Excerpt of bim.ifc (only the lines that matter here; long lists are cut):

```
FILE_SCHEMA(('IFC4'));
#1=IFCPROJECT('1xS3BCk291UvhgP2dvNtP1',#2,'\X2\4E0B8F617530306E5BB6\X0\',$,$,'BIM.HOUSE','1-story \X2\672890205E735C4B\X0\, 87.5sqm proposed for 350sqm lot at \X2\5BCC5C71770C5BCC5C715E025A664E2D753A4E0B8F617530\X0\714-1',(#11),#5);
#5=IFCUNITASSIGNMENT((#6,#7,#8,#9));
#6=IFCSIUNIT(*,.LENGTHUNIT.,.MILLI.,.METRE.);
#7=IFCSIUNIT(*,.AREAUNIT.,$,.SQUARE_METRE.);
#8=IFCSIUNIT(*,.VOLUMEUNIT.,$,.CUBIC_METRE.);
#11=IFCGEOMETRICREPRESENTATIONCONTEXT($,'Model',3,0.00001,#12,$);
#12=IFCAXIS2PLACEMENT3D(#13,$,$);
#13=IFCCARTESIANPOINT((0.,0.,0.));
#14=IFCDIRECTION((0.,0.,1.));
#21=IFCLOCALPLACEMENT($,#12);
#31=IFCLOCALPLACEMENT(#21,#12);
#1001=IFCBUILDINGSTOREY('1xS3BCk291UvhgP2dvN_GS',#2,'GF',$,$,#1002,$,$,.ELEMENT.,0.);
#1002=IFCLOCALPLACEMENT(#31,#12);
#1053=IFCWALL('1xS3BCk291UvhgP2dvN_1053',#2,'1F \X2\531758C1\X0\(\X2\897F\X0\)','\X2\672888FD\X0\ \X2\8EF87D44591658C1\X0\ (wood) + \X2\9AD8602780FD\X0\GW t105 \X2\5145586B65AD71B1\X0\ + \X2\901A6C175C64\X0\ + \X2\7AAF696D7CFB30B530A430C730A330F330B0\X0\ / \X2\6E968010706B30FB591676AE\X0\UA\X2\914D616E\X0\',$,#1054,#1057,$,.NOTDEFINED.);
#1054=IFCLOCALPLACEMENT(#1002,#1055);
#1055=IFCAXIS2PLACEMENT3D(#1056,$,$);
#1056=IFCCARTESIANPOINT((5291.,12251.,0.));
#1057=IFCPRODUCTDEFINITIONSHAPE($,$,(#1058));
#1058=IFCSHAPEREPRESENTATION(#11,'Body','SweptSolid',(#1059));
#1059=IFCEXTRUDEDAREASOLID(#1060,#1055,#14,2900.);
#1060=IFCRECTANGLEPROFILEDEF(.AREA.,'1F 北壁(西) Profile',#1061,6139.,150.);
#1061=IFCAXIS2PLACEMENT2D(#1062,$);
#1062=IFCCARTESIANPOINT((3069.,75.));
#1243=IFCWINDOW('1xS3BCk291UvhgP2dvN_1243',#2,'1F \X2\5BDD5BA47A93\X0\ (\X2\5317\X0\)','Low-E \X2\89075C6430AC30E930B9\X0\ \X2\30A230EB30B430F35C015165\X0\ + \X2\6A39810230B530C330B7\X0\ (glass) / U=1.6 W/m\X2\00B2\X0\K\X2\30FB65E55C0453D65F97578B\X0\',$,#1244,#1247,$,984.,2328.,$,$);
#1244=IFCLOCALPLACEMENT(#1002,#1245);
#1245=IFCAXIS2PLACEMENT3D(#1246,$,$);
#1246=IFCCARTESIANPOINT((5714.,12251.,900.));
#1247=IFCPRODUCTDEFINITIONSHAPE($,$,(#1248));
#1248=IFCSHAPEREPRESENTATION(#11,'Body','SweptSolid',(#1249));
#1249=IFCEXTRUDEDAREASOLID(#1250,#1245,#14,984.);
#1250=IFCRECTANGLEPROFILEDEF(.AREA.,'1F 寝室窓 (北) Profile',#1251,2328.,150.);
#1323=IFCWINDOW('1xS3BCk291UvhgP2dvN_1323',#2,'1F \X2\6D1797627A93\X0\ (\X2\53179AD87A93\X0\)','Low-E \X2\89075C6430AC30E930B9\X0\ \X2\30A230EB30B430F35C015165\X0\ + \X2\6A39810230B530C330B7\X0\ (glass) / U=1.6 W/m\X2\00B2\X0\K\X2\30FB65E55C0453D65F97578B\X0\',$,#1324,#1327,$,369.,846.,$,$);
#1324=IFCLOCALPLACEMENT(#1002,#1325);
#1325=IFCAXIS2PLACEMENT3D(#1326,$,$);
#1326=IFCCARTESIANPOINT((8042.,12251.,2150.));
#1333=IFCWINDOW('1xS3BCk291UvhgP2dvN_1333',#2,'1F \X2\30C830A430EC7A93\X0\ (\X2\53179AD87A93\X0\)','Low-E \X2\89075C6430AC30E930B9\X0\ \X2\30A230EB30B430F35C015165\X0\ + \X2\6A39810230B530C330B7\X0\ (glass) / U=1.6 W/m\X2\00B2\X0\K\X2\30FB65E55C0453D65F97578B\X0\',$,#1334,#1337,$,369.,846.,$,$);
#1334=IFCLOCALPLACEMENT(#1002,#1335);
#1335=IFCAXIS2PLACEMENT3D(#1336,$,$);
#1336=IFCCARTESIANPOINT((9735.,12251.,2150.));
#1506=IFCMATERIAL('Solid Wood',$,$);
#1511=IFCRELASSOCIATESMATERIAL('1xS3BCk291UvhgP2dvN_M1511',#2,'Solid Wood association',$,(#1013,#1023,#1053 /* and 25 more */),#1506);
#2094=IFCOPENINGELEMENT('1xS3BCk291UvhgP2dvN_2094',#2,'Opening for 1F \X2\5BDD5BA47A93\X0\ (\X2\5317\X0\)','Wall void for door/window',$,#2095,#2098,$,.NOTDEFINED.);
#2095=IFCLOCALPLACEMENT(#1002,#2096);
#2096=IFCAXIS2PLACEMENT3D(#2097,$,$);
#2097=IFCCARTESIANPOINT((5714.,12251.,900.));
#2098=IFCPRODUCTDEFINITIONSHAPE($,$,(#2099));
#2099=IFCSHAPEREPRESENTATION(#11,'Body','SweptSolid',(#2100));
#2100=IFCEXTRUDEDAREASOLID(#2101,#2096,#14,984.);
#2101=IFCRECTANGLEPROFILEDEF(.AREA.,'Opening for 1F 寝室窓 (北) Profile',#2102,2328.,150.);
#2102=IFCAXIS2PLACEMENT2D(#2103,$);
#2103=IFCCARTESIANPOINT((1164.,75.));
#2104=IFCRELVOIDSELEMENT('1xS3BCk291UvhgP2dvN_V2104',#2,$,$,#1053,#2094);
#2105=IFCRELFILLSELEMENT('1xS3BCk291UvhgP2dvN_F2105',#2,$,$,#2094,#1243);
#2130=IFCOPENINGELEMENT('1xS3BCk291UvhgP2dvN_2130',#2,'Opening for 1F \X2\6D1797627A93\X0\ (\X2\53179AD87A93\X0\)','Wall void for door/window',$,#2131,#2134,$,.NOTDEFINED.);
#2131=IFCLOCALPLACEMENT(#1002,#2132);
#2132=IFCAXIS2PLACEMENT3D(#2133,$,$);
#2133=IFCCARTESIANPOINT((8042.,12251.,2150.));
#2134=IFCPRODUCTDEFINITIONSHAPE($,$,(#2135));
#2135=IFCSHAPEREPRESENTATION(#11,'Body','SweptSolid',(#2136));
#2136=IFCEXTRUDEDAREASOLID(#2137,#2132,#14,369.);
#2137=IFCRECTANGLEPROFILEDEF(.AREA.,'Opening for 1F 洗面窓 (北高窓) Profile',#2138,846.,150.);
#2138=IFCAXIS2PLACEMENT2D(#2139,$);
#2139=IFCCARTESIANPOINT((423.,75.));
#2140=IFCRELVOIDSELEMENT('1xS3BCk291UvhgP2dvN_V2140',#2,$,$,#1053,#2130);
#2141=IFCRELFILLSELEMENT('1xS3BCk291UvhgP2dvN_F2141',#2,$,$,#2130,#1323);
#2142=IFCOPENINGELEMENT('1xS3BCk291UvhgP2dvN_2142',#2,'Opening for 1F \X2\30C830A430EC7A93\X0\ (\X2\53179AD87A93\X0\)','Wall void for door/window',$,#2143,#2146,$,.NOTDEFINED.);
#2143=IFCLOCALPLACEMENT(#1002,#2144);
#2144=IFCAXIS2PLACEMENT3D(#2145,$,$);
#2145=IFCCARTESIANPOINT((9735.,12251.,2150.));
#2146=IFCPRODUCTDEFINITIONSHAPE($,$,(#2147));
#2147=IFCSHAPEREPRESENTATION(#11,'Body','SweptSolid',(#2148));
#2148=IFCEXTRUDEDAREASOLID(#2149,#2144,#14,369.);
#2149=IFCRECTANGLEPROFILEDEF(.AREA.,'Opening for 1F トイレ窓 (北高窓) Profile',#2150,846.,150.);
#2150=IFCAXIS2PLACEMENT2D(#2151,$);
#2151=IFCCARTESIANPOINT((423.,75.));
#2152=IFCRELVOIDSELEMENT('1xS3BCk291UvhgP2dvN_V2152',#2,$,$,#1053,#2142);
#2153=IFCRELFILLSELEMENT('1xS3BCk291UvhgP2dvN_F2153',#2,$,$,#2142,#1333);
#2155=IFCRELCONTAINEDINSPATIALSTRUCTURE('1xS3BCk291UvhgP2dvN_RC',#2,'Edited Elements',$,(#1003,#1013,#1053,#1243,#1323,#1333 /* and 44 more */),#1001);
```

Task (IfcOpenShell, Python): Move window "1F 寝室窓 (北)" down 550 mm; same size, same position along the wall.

```python
import numpy as np
import ifcopenshell
import ifcopenshell.api.geometry
import ifcopenshell.util.placement
import ifcopenshell.util.unit

model = ifcopenshell.open("bim.ifc")
unit_scale = ifcopenshell.util.unit.calculate_unit_scale(model)

window = model.by_id(1243)
opening = window.FillsVoids[0].RelatingOpeningElement
dz = -550.0

shift = np.array([0.0, 0.0, dz])
# The window is not placed relative to its opening, so move both.
for product in (opening, window):
    matrix = ifcopenshell.util.placement.get_local_placement(product.ObjectPlacement)
    matrix[:3, 3] += shift
    ifcopenshell.api.geometry.edit_object_placement(model, product=product, matrix=matrix, is_si=False)

print(f"moved by {dz * unit_scale:+.3f} m")

model.write("bim-out.ifc")
```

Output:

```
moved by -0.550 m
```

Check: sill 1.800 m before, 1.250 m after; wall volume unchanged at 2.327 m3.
